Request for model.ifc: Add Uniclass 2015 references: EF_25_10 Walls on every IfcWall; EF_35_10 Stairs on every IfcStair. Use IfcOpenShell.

First a look at what the model holds.

```python
import ifcopenshell

model = ifcopenshell.open("model.ifc")
print(model.schema)
print("classifications:", [c.Name for c in model.by_type("IfcClassification")])
for ifc_class in ("IfcDoor", "IfcRoof", "IfcStair", "IfcWall", "IfcWindow"):
    print(ifc_class, len(model.by_type(ifc_class)))
```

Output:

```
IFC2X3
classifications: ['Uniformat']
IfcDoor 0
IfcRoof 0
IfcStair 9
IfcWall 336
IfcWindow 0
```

```python
import ifcopenshell
import ifcopenshell.api.classification

model = ifcopenshell.open("model.ifc")

# IFC2X3 requires Source and Edition and has no link from the project to the system.
system = model.create_entity("IfcClassification", Source="NBS", Edition="2015", Name="Uniclass 2015")

codes = {
    "IfcWall": ("EF_25_10", "Walls"),
    "IfcStair": ("EF_35_10", "Stairs"),
}
for ifc_class, (code, name) in codes.items():
    products = model.by_type(ifc_class)
    ifcopenshell.api.classification.add_reference(
        model, products=products, classification=system, identification=code, name=name
    )
    print(code, len(products))

model.write("model-out.ifc")
```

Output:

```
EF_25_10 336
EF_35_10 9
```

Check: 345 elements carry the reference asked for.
